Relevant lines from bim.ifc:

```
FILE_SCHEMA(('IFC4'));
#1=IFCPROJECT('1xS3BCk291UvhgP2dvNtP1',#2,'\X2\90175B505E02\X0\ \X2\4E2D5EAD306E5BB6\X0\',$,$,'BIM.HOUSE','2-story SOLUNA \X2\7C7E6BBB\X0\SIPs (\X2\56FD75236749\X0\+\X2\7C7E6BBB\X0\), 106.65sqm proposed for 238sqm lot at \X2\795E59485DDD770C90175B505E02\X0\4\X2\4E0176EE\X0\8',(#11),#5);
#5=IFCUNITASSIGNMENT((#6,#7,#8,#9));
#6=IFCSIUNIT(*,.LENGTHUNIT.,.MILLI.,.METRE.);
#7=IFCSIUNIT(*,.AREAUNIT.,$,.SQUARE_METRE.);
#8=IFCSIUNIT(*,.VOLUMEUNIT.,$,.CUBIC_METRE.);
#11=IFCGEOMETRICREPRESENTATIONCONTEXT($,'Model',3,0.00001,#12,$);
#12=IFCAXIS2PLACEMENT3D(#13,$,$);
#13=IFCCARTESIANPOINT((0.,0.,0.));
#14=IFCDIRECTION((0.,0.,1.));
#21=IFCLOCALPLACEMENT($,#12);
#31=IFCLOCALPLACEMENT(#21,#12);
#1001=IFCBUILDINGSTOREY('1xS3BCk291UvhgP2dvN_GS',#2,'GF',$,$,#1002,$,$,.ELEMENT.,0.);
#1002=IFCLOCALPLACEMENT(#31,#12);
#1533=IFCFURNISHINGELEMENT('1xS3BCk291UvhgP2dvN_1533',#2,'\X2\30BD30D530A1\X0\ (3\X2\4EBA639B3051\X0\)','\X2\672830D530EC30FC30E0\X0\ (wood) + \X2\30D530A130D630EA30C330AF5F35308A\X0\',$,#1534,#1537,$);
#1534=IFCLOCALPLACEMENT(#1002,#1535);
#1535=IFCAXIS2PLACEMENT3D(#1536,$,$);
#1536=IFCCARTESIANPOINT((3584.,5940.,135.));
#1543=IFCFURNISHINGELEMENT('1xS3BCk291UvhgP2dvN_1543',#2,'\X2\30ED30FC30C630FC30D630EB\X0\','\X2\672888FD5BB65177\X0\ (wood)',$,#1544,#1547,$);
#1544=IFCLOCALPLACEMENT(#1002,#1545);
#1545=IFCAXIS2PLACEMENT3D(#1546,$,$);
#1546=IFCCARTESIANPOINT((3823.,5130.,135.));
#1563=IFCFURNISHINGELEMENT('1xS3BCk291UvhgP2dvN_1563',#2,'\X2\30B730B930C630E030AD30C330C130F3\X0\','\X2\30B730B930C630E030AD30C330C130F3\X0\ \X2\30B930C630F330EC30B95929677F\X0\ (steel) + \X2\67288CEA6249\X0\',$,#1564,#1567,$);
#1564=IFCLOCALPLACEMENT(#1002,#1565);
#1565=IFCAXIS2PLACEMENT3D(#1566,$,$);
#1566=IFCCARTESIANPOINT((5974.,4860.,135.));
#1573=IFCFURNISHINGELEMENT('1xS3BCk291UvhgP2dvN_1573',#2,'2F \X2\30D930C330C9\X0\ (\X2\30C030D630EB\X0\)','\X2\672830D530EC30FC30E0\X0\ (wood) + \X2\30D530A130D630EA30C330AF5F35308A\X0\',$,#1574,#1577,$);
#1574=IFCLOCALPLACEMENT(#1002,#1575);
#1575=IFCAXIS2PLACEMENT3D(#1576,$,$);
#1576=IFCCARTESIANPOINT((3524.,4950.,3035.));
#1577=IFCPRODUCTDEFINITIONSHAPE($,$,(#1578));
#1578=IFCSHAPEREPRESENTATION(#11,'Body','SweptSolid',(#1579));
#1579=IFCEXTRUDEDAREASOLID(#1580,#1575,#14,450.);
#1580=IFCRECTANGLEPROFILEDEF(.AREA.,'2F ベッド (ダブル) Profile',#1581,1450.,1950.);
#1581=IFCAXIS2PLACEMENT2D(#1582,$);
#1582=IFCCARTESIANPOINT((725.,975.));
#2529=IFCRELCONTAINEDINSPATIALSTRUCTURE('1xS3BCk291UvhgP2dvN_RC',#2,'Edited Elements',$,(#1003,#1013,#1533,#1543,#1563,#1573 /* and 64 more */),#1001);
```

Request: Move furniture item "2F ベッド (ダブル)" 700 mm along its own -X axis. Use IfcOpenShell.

```python
import ifcopenshell
import ifcopenshell.api.geometry
import ifcopenshell.util.placement
import ifcopenshell.util.unit

model = ifcopenshell.open("bim.ifc")
unit_scale = ifcopenshell.util.unit.calculate_unit_scale(model)

item = model.by_guid("1xS3BCk291UvhgP2dvN_1573")
matrix = ifcopenshell.util.placement.get_local_placement(item.ObjectPlacement)
matrix[:3, 3] -= matrix[:3, 0] * 0.7 / unit_scale
ifcopenshell.api.geometry.edit_object_placement(model, product=item, matrix=matrix, is_si=False)

print(ifcopenshell.util.placement.get_local_placement(item.ObjectPlacement).round(3) + 0.0)

model.write("bim_edited.ifc")
```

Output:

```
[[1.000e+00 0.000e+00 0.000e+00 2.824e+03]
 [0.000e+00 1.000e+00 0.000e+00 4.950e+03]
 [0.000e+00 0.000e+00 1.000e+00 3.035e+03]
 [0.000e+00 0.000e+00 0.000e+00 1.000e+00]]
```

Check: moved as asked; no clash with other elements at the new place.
